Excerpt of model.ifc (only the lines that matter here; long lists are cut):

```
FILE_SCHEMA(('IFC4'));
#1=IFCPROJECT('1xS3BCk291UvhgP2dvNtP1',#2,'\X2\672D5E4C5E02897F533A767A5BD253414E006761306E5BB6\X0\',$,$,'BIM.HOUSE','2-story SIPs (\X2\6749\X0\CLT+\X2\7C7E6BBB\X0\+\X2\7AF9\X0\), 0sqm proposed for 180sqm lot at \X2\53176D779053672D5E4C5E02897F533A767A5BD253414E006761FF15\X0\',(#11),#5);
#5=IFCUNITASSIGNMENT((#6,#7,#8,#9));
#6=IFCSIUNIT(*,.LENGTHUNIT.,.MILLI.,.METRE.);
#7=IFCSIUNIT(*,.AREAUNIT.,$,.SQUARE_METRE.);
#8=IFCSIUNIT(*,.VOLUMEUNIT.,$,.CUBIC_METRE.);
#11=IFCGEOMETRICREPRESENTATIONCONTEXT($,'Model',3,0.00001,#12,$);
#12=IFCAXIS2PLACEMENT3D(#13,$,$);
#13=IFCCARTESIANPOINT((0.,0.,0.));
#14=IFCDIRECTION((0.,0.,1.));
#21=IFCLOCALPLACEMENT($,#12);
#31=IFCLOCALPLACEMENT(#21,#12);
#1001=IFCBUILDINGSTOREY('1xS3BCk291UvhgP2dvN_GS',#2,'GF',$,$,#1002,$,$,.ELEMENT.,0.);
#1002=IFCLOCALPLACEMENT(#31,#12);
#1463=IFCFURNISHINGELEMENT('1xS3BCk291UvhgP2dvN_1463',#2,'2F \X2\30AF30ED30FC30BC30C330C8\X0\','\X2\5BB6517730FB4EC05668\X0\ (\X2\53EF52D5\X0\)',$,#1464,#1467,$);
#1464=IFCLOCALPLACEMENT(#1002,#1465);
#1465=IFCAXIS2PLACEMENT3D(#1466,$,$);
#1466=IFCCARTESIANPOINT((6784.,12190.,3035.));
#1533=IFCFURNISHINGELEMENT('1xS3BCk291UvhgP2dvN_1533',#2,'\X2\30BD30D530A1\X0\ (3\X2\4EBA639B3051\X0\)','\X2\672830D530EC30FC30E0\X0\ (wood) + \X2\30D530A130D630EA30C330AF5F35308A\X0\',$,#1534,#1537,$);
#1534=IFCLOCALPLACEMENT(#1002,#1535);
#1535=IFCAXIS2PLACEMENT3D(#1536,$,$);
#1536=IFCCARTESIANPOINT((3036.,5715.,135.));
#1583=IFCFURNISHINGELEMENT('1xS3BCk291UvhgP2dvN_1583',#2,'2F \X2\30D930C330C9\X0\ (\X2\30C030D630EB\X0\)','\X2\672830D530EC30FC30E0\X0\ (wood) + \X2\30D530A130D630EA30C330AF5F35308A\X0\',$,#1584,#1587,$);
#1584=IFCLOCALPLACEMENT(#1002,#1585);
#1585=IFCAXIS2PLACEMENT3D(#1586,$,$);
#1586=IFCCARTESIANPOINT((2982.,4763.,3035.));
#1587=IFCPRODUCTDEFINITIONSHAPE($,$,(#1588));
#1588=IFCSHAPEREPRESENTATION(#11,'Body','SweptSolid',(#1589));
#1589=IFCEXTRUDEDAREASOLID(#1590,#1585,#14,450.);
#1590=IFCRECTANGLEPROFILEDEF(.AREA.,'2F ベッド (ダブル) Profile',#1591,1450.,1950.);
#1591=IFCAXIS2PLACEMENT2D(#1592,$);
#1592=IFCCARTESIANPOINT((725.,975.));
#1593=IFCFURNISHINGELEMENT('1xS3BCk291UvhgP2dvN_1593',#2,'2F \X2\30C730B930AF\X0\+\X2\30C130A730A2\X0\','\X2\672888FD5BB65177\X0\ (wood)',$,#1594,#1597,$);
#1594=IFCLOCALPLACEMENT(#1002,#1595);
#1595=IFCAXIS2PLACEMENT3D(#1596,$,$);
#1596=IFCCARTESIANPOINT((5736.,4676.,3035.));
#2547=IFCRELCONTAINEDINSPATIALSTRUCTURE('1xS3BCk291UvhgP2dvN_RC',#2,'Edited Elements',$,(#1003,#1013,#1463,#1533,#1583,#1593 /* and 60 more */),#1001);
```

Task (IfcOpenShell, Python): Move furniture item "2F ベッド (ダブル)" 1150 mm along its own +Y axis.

```python
import ifcopenshell
import ifcopenshell.api.geometry
import ifcopenshell.util.placement
import ifcopenshell.util.unit

model = ifcopenshell.open("model.ifc")
unit_scale = ifcopenshell.util.unit.calculate_unit_scale(model)

item = model.by_id(1583)
matrix = ifcopenshell.util.placement.get_local_placement(item.ObjectPlacement)
matrix[:3, 3] += matrix[:3, 1] * 1.15 / unit_scale
ifcopenshell.api.geometry.edit_object_placement(model, product=item, matrix=matrix, is_si=False)

print(ifcopenshell.util.placement.get_local_placement(item.ObjectPlacement).round(3) + 0.0)

model.write("model_edited.ifc")
```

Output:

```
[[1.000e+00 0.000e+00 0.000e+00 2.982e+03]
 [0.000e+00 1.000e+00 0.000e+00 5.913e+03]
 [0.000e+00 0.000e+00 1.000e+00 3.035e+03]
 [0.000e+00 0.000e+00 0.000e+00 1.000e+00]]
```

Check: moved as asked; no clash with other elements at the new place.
